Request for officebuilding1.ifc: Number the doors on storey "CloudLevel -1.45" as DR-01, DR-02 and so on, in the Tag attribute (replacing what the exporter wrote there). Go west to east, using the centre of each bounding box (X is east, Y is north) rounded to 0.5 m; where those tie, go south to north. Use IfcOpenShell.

First a look at what the model holds.

```python
import ifcopenshell
import ifcopenshell.util.element
import ifcopenshell.util.placement

model = ifcopenshell.open("officebuilding1.ifc")
print(model.schema)
storey = next(s for s in model.by_type("IfcBuildingStorey") if s.Name == "CloudLevel -1.45")
doors = [e for e in ifcopenshell.util.element.get_decomposition(storey) if e.is_a("IfcDoor")]
for e in sorted(doors, key=lambda e: e.id()):
    origin = ifcopenshell.util.placement.get_local_placement(e.ObjectPlacement)[:3, 3]
    print(e.id(), e.Tag, e.Name, origin.round(2) + 0.0, sep=" | ")
```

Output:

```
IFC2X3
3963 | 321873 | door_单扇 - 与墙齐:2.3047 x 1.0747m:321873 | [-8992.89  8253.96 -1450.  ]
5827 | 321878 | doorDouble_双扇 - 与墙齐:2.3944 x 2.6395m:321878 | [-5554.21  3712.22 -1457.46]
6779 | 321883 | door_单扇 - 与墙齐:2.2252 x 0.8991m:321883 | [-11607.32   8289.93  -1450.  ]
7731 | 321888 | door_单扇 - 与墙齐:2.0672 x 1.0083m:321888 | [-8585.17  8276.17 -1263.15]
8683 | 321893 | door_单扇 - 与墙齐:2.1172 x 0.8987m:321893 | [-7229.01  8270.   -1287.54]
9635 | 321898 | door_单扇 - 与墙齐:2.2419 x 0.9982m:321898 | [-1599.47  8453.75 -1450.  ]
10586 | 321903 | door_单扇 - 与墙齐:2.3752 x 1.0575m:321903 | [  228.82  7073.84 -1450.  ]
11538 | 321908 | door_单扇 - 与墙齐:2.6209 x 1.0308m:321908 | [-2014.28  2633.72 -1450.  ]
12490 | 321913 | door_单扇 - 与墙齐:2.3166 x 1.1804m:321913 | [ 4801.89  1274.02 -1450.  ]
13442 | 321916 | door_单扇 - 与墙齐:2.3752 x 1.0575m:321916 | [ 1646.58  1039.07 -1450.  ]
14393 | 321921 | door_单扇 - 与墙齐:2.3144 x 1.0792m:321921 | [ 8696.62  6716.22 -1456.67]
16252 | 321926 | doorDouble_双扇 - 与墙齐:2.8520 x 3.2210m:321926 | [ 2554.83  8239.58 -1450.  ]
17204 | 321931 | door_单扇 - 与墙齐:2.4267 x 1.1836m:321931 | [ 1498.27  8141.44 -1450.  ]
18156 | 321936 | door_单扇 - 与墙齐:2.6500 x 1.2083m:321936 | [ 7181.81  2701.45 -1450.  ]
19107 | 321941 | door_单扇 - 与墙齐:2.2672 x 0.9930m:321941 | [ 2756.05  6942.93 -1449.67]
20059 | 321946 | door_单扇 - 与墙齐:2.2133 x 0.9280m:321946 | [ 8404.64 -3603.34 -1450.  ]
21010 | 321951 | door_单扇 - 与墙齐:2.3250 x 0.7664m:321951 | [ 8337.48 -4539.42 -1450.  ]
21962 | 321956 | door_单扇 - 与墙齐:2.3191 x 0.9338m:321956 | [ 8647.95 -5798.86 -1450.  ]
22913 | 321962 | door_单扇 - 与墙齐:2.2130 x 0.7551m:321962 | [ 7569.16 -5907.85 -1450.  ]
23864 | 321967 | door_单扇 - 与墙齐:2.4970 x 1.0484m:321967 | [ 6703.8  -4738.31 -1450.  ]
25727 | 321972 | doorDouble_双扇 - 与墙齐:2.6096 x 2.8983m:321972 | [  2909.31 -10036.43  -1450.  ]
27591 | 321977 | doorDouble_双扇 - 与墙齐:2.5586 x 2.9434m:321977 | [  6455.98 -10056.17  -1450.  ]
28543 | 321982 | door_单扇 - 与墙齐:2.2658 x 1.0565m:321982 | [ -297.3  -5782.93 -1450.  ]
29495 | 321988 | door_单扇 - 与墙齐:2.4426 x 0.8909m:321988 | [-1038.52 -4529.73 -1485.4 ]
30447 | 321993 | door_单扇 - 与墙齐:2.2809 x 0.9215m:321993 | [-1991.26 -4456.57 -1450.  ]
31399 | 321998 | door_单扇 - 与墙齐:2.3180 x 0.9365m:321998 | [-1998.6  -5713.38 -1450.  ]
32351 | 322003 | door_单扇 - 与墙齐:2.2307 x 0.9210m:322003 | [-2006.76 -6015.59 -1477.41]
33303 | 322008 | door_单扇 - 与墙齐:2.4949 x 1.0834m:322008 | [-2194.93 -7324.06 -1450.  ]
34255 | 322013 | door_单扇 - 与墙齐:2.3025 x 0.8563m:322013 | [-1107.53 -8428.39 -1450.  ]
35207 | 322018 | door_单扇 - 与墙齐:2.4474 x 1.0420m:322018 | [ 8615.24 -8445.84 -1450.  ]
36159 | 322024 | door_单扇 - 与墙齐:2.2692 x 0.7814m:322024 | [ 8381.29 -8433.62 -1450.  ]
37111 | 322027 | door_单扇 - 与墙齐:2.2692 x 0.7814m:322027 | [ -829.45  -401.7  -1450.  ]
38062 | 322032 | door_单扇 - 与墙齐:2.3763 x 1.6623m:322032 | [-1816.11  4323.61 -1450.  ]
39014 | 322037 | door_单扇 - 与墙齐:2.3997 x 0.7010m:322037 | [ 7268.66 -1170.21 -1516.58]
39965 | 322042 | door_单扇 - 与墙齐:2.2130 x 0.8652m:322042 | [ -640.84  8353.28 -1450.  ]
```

```python
import ifcopenshell
import ifcopenshell.geom
import ifcopenshell.util.element
import ifcopenshell.util.shape

model = ifcopenshell.open("officebuilding1.ifc")
settings = ifcopenshell.geom.settings()
settings.set("use-world-coords", True)


def centre(element):
    shape = ifcopenshell.geom.create_shape(settings, element)
    return ifcopenshell.util.shape.get_bbox_centroid(shape.geometry)


storey = next(s for s in model.by_type("IfcBuildingStorey") if s.Name == "CloudLevel -1.45")
doors = [e for e in ifcopenshell.util.element.get_decomposition(storey) if e.is_a("IfcDoor")]

# Insertion points can sit at a corner or the storey origin, so sort by the geometry (in metres).
centres = {e: centre(e) for e in doors}
doors.sort(key=lambda e: (round(centres[e][0] / 0.5), centres[e][1]))

for i, e in enumerate(doors, start=1):
    number = f"DR-{i:02d}"
    e.Tag = number
    print(e.id(), number)

model.write("officebuilding1_v2.ifc")
```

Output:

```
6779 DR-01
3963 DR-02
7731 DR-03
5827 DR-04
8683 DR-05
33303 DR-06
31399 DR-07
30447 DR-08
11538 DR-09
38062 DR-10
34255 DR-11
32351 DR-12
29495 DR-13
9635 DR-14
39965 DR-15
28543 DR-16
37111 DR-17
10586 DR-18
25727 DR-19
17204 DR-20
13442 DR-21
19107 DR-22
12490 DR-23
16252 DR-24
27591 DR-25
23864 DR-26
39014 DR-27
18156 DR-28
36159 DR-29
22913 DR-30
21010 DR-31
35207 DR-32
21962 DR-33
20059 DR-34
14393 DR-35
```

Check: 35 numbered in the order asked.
